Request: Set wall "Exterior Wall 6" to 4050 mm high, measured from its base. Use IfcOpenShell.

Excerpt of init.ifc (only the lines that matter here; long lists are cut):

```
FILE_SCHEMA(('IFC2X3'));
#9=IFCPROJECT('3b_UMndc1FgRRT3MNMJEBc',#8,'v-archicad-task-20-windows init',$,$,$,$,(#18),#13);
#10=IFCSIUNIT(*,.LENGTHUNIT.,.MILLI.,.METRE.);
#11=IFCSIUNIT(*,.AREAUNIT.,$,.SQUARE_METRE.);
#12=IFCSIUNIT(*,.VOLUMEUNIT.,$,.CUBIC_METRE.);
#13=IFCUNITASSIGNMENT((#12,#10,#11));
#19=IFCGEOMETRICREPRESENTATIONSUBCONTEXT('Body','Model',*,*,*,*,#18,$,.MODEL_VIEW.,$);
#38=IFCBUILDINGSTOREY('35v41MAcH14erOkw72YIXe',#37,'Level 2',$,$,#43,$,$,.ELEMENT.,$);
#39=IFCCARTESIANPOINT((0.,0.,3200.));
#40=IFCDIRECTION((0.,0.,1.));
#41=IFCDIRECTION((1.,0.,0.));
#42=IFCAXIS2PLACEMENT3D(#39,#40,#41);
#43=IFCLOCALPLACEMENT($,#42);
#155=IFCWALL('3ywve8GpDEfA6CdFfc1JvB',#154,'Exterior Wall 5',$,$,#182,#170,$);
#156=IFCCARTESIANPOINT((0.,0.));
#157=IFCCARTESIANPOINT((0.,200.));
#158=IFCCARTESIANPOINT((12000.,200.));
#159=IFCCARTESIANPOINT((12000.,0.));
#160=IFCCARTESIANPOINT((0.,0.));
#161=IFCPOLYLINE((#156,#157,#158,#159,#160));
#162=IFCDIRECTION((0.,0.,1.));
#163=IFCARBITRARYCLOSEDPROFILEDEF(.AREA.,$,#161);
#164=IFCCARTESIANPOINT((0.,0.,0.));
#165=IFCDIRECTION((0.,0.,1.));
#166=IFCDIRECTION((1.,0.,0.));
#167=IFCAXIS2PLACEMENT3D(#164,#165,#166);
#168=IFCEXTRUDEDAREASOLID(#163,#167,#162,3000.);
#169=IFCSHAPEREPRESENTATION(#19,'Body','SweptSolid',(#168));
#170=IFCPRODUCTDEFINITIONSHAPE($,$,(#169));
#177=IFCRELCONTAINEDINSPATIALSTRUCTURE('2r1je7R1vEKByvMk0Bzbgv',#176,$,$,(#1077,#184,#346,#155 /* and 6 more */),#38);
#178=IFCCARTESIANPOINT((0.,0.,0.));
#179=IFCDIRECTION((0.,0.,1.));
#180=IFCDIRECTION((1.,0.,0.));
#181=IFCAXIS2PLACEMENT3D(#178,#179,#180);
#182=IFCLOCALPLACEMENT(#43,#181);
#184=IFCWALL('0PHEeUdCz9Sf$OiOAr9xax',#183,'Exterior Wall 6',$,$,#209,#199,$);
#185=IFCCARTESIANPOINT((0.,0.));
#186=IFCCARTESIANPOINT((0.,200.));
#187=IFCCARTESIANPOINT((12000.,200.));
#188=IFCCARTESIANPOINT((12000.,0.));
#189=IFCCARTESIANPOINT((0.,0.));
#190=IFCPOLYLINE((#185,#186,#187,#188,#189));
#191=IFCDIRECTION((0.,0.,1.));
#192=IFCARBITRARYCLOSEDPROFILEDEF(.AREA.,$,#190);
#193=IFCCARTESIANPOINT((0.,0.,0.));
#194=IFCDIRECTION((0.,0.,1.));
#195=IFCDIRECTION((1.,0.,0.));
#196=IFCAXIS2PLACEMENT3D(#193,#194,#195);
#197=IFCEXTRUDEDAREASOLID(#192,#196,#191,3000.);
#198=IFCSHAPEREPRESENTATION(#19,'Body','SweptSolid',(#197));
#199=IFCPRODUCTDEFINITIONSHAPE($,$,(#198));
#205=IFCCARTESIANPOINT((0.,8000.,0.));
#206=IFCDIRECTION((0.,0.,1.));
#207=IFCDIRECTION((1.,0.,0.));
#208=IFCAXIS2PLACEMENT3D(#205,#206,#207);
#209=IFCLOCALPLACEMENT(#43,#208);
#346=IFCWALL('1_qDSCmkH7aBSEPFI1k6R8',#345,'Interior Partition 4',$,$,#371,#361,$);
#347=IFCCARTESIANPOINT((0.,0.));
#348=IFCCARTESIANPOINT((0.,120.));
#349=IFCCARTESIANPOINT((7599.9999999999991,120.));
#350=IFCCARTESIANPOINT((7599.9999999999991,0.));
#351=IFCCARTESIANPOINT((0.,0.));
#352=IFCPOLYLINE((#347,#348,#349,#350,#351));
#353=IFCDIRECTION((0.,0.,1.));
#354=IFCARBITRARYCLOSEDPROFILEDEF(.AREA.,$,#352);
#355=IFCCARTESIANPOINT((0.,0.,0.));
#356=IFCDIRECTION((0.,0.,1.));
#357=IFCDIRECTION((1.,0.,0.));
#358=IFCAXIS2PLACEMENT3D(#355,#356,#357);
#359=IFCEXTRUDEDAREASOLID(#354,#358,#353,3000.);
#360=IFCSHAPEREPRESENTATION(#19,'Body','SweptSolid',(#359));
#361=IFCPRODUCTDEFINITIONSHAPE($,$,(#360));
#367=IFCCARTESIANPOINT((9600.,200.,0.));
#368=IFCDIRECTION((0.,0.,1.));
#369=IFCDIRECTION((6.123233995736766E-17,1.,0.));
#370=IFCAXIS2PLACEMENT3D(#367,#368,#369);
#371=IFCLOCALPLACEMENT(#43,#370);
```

```python
import ifcopenshell
import ifcopenshell.geom
import ifcopenshell.util.representation
import ifcopenshell.util.shape

model = ifcopenshell.open("init.ifc")
settings = ifcopenshell.geom.settings()


def volume(element):
    """Net volume in cubic metres, openings subtracted."""
    shape = ifcopenshell.geom.create_shape(settings, element)
    return ifcopenshell.util.shape.get_volume(shape.geometry)


wall = model.by_id(184)
before = volume(wall)

body = ifcopenshell.util.representation.get_representation(wall, "Model", "Body")
solid = body.Items[0]
old_height = solid.Depth
solid.Depth = 4050.0
after = volume(wall)

print(f"height {old_height:g} -> {solid.Depth:g}, volume {before:.3f} -> {after:.3f} m3")

model.write("init-out.ifc")
```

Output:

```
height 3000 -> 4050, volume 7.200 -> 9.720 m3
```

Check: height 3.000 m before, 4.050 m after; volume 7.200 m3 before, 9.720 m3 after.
